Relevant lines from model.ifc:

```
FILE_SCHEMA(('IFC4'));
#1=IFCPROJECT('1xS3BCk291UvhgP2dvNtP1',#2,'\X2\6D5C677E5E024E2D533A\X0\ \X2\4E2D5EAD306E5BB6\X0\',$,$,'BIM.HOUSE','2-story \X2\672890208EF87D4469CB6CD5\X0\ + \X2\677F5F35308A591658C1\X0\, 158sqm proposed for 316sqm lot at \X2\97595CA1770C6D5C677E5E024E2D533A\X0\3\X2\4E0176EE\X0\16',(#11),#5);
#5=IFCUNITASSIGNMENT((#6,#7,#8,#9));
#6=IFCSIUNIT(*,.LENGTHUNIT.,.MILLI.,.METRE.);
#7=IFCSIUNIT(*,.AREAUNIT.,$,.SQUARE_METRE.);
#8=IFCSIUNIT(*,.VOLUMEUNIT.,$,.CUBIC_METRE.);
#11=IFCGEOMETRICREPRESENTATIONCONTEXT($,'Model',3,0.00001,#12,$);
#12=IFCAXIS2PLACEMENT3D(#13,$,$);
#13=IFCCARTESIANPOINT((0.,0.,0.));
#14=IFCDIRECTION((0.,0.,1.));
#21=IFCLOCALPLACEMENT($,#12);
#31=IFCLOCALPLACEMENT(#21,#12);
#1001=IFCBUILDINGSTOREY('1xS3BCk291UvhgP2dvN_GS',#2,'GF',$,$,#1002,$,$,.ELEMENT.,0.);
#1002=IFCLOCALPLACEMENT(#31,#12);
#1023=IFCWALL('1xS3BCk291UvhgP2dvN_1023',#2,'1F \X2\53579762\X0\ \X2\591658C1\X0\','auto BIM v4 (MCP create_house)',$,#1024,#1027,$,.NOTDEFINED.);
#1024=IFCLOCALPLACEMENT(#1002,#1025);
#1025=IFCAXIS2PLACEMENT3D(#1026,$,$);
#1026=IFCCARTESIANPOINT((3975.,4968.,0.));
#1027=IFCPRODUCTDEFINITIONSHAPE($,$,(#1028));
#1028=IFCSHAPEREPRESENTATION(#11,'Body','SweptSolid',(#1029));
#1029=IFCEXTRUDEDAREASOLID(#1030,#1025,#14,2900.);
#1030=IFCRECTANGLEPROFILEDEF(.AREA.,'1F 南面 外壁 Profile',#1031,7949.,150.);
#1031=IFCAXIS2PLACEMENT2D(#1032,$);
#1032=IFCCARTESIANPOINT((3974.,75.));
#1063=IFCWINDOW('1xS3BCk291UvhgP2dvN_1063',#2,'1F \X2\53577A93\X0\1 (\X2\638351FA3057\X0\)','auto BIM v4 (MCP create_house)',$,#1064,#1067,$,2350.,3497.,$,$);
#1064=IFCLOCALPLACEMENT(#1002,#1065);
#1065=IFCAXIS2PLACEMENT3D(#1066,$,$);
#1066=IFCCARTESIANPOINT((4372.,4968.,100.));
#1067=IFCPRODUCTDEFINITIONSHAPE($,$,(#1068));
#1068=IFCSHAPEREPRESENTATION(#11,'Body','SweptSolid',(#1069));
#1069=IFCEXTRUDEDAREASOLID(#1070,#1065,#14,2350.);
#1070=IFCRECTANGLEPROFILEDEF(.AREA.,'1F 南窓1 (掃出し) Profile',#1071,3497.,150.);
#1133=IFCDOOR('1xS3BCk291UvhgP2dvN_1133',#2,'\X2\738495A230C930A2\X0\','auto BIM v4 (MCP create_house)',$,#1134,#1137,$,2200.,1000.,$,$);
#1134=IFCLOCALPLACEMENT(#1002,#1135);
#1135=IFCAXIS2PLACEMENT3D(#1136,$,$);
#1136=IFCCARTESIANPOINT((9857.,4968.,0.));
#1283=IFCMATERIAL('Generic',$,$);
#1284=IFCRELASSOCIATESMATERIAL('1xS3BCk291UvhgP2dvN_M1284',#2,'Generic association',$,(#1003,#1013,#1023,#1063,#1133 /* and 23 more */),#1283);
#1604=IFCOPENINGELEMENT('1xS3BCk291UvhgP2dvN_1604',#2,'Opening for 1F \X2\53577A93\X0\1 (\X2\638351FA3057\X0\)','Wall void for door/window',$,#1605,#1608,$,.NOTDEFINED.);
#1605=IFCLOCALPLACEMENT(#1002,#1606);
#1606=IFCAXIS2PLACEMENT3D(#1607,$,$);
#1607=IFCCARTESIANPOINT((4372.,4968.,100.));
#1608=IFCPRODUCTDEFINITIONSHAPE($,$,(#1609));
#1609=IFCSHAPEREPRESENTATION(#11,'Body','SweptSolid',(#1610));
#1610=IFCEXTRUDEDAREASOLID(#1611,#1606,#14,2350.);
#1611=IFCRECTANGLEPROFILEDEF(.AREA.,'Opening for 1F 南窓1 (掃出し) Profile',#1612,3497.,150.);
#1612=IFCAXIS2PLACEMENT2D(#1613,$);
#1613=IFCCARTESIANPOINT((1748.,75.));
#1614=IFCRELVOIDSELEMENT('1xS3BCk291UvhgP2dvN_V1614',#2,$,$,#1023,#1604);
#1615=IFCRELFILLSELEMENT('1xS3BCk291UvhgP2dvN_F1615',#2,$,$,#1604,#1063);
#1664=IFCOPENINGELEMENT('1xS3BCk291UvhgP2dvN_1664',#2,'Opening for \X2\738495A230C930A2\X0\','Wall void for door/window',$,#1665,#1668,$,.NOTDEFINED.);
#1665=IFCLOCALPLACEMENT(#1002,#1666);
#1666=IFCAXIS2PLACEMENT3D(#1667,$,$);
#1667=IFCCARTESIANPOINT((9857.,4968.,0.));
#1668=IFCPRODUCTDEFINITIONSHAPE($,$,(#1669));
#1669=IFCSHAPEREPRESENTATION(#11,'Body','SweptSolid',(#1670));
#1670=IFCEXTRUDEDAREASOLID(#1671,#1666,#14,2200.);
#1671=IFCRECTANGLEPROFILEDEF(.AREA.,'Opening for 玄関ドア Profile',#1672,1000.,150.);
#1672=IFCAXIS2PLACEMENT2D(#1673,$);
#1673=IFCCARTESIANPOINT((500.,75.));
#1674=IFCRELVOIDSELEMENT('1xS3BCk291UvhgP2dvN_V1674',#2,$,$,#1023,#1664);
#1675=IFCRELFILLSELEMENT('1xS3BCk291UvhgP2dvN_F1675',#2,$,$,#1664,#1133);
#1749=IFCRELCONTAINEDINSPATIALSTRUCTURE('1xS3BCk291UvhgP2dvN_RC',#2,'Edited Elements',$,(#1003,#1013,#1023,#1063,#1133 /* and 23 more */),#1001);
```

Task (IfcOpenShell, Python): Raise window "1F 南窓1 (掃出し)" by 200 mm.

```python
import numpy as np
import ifcopenshell
import ifcopenshell.api.geometry
import ifcopenshell.util.placement
import ifcopenshell.util.unit

model = ifcopenshell.open("model.ifc")
unit_scale = ifcopenshell.util.unit.calculate_unit_scale(model)

window = model.by_guid("1xS3BCk291UvhgP2dvN_1063")
opening = window.FillsVoids[0].RelatingOpeningElement
dz = 0.2 / unit_scale

shift = np.array([0.0, 0.0, dz])
# The window is not placed relative to its opening, so move both.
for product in (opening, window):
    matrix = ifcopenshell.util.placement.get_local_placement(product.ObjectPlacement)
    matrix[:3, 3] += shift
    ifcopenshell.api.geometry.edit_object_placement(model, product=product, matrix=matrix, is_si=False)

print(f"moved by {dz * unit_scale:+.3f} m")

model.write("model_updated.ifc")
```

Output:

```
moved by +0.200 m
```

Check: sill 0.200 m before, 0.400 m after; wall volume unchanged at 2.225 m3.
